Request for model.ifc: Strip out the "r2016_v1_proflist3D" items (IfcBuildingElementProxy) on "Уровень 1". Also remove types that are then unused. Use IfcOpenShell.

First a look at what the model holds.

```python
import ifcopenshell
import ifcopenshell.util.element

model = ifcopenshell.open("model.ifc")
print(model.schema)
storey = next(s for s in model.by_type("IfcBuildingStorey") if s.Name == "Уровень 1")
proxies = [e for e in ifcopenshell.util.element.get_decomposition(storey) if e.is_a("IfcBuildingElementProxy")]
seen = {}
for e in proxies:
    element_type = ifcopenshell.util.element.get_type(e)
    name = element_type.Name if element_type not in (None, e) else None
    seen[name] = seen.get(name, 0) + 1
for name, count in sorted(seen.items(), key=str):
    print(count, "x", name)
```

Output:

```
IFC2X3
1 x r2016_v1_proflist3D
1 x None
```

```python
import ifcopenshell
import ifcopenshell.api.root
import ifcopenshell.util.element

model = ifcopenshell.open("model.ifc")

storey = next(s for s in model.by_type("IfcBuildingStorey") if s.Name == "Уровень 1")
proxies = [e for e in ifcopenshell.util.element.get_decomposition(storey) if e.is_a("IfcBuildingElementProxy")]
targets = [e for e in proxies if (t := ifcopenshell.util.element.get_type(e)) not in (None, e) and t.Name == "r2016_v1_proflist3D"]
types = {ifcopenshell.util.element.get_type(e) for e in targets} - {None, *targets}

for e in targets:
    ifcopenshell.api.root.remove_product(model, product=e)
print(len(targets), "removed")

unused = [t for t in types if not ifcopenshell.util.element.get_types(t)]
for t in unused:
    ifcopenshell.api.root.remove_product(model, product=t)
print(len(unused), "unused types removed")

model.write("model_v2.ifc")
```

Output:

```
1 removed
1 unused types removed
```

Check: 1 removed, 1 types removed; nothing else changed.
